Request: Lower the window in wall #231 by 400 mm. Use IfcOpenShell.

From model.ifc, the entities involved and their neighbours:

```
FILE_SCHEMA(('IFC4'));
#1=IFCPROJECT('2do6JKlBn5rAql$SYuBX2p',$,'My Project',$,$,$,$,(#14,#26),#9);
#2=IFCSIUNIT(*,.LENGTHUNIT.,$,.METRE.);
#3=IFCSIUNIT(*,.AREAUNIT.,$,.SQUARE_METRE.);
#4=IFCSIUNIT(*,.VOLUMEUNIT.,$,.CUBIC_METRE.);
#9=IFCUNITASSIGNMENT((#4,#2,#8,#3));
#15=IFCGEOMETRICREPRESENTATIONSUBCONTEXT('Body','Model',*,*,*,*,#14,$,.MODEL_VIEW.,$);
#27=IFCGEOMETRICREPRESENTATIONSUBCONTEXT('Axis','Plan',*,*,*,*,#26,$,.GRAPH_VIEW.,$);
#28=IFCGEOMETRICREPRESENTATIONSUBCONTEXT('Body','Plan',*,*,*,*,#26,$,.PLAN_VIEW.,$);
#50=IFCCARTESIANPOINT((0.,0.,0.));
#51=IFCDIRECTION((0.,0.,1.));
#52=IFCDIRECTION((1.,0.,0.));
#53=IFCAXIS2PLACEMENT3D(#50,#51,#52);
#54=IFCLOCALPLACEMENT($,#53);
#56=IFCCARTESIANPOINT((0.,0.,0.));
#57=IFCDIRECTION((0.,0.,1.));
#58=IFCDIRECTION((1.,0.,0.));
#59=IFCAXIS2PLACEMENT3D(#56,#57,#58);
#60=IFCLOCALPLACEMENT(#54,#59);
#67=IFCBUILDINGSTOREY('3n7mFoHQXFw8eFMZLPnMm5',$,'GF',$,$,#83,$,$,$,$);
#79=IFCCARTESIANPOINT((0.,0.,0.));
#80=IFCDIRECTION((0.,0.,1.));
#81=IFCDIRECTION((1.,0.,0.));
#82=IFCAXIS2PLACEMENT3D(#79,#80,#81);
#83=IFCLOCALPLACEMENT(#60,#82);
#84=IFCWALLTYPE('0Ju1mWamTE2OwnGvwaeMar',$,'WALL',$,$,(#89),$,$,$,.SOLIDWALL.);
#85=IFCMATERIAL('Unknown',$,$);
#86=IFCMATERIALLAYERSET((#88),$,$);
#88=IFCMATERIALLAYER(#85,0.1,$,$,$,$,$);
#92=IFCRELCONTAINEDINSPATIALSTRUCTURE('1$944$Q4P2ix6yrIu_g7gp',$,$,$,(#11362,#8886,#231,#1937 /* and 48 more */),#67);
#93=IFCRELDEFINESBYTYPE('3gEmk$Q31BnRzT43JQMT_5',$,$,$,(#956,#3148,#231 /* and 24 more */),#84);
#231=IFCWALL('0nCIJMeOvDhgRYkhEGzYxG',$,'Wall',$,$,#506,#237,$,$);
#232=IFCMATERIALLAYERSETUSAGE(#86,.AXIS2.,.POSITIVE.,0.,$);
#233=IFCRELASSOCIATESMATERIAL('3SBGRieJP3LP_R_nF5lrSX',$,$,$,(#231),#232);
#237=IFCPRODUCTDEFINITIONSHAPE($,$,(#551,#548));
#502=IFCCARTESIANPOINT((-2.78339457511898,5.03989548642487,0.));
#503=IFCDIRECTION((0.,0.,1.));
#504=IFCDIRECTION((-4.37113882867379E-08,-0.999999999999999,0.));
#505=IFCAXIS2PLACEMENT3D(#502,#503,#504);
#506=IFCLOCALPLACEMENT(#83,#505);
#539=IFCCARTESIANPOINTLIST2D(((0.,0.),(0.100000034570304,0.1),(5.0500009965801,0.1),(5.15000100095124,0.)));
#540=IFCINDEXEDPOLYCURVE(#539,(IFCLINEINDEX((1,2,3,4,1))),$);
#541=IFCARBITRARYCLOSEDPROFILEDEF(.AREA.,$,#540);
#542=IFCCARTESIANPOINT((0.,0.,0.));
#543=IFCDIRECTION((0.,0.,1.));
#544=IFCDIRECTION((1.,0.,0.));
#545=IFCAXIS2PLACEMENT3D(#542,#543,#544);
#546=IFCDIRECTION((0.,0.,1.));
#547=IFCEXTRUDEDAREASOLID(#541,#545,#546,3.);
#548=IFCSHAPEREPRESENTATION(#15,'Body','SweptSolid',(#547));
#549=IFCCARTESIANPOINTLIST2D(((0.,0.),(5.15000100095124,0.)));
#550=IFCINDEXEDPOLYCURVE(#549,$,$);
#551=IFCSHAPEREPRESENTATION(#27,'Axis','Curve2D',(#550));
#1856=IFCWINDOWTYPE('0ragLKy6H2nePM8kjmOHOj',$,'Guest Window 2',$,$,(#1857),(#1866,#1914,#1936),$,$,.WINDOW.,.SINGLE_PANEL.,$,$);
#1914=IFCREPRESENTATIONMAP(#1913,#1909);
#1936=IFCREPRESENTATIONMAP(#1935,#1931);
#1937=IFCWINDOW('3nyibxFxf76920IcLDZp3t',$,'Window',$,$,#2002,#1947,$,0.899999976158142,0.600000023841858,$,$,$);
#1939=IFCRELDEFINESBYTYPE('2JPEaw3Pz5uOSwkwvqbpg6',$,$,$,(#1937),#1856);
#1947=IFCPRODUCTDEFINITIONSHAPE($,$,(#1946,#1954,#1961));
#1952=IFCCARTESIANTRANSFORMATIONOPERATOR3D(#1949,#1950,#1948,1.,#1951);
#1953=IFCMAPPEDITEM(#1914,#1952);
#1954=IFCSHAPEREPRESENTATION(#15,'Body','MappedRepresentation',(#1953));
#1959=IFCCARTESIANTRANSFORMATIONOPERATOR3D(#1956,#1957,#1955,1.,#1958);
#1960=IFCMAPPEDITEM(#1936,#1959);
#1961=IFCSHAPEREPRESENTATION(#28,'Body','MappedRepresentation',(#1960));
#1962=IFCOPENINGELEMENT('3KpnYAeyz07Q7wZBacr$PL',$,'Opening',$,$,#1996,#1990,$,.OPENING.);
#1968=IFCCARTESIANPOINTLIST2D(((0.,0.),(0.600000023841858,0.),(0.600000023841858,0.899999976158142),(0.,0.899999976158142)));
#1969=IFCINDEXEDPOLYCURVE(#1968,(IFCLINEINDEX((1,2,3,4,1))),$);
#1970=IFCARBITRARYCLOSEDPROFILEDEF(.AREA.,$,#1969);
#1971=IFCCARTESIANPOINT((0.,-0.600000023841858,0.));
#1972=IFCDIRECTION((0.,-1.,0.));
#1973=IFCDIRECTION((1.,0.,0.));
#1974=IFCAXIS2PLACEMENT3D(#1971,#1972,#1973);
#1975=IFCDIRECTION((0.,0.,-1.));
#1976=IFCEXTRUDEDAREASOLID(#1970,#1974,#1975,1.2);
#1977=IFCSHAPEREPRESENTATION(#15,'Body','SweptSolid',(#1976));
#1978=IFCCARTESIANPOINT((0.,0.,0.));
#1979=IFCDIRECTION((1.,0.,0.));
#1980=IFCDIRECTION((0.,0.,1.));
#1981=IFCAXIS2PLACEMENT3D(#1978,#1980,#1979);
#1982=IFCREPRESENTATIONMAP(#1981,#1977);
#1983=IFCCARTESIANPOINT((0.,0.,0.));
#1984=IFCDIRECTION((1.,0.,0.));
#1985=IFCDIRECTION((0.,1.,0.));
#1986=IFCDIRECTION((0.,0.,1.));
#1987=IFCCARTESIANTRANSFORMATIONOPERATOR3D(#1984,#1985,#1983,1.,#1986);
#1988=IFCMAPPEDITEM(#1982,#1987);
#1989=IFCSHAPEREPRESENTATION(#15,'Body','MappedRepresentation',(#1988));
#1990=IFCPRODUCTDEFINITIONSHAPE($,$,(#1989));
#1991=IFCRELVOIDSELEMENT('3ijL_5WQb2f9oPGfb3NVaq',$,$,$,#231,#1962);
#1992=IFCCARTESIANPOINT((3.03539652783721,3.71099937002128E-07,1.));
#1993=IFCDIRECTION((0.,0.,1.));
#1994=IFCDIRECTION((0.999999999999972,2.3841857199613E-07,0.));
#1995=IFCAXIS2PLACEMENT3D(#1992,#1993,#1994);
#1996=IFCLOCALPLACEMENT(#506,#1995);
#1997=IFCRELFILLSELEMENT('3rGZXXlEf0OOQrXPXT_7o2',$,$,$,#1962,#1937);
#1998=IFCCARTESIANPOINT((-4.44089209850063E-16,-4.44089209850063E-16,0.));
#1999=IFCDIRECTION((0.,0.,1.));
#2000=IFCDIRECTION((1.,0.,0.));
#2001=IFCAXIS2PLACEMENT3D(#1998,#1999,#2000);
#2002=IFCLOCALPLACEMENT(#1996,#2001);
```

```python
import numpy as np
import ifcopenshell
import ifcopenshell.api.geometry
import ifcopenshell.util.placement
import ifcopenshell.util.unit

model = ifcopenshell.open("model.ifc")
unit_scale = ifcopenshell.util.unit.calculate_unit_scale(model)

window = model.by_guid("3nyibxFxf76920IcLDZp3t")
opening = window.FillsVoids[0].RelatingOpeningElement
dz = -0.4 / unit_scale

shift = np.array([0.0, 0.0, dz])
# The window is placed relative to its opening, so it follows when the opening moves.
matrix = ifcopenshell.util.placement.get_local_placement(opening.ObjectPlacement)
matrix[:3, 3] += shift
ifcopenshell.api.geometry.edit_object_placement(
    model, product=opening, matrix=matrix, is_si=False, should_transform_children=True
)

print(f"moved by {dz * unit_scale:+.3f} m")

model.write("model_edited.ifc")
```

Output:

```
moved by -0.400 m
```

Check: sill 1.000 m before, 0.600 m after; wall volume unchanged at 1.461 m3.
